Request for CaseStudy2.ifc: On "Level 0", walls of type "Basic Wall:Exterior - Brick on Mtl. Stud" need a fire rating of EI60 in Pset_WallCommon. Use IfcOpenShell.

First a look at what the model holds.

```python
import ifcopenshell
import ifcopenshell.util.element

model = ifcopenshell.open("CaseStudy2.ifc")
print(model.schema)
storey = next(s for s in model.by_type("IfcBuildingStorey") if s.Name == "Level 0")
walls = [e for e in ifcopenshell.util.element.get_decomposition(storey) if e.is_a("IfcWall")]
seen = {}
for e in walls:
    element_type = ifcopenshell.util.element.get_type(e)
    key = (element_type.Name if element_type != e and element_type else None, ifcopenshell.util.element.get_pset(e, "Pset_WallCommon", "FireRating"))
    seen[key] = seen.get(key, 0) + 1
for (name, value), count in sorted(seen.items(), key=str):
    print(count, "x", name, "|", value)
```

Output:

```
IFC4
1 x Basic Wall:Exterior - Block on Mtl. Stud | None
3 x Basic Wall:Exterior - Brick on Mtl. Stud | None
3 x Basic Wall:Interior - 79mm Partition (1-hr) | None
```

```python
import ifcopenshell
import ifcopenshell.api.pset
import ifcopenshell.util.element

model = ifcopenshell.open("CaseStudy2.ifc")

storey = next(s for s in model.by_type("IfcBuildingStorey") if s.Name == "Level 0")
walls = [e for e in ifcopenshell.util.element.get_decomposition(storey) if e.is_a("IfcWall")]

count = 0
for e in walls:
    element_type = ifcopenshell.util.element.get_type(e)
    if element_type in (None, e) or element_type.Name != "Basic Wall:Exterior - Brick on Mtl. Stud":
        continue
    # add_pset returns the element's existing set when there is one.
    pset = ifcopenshell.api.pset.add_pset(model, product=e, name="Pset_WallCommon")
    ifcopenshell.api.pset.edit_pset(model, pset=pset, properties={"FireRating": "EI60"})
    count += 1

print(count, "walls updated")

model.write("CaseStudy2_updated.ifc")
```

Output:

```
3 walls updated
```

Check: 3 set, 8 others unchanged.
